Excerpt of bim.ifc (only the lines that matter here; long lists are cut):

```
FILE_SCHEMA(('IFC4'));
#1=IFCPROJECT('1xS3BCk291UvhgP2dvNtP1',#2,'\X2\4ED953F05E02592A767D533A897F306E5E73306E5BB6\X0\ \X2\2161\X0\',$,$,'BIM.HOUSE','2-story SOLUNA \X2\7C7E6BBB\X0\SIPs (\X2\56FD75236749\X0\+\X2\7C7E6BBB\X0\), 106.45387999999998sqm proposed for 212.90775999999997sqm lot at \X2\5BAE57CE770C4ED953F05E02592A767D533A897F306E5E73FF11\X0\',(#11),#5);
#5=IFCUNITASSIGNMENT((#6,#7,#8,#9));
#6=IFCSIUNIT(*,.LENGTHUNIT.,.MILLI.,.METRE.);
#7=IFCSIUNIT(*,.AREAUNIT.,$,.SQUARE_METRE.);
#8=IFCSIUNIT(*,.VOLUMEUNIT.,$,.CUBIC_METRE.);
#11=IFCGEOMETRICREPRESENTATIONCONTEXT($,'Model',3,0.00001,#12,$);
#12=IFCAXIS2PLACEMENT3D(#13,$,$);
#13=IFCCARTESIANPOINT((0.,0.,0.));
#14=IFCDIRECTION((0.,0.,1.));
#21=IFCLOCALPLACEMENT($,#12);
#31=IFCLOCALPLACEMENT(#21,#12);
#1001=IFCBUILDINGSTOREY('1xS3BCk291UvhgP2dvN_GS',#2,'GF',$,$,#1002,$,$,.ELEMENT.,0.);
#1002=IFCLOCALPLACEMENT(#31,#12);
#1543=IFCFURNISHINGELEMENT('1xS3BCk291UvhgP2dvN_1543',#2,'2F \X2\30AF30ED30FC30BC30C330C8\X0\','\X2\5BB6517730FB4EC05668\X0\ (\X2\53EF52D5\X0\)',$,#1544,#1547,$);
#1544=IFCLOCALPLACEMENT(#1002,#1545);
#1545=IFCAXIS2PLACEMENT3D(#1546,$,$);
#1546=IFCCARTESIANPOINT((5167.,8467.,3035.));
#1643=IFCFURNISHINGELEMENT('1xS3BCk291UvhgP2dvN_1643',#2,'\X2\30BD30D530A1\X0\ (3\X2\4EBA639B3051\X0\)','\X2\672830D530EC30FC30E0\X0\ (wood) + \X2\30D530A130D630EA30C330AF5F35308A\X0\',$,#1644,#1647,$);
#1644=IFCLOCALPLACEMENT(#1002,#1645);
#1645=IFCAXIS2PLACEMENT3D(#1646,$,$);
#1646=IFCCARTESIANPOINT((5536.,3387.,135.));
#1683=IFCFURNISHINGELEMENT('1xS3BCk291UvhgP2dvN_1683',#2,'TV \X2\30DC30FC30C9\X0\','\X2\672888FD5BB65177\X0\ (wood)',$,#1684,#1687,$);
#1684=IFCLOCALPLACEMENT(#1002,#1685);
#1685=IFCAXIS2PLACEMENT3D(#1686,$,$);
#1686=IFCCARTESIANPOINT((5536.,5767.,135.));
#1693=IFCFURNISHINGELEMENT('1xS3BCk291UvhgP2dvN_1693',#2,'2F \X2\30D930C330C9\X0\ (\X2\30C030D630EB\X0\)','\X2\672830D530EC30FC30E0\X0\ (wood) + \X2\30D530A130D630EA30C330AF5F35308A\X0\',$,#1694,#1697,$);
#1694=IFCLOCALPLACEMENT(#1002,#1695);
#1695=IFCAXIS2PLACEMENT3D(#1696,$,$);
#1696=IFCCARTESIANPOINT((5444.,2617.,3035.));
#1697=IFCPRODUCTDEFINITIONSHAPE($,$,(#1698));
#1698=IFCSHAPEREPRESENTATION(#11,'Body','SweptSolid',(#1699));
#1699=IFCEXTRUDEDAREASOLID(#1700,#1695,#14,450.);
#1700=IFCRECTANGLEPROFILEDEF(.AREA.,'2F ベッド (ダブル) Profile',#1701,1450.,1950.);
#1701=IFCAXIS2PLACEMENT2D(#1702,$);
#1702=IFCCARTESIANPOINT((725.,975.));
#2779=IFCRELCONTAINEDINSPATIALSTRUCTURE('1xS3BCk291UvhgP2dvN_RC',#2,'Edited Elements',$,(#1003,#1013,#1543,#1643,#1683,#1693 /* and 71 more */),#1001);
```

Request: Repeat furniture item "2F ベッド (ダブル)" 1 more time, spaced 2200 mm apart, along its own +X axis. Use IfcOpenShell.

```python
import ifcopenshell
import ifcopenshell.api.geometry
import ifcopenshell.api.root
import ifcopenshell.util.element
import ifcopenshell.util.placement

model = ifcopenshell.open("bim.ifc")


def reuse_history(source, copy):
    """copy_class also copies each property set's owner history, people and application; keep the originals."""
    for rel in copy.IsDefinedBy:
        if rel.is_a("IfcRelDefinesByProperties") and (history := rel.RelatingPropertyDefinition.OwnerHistory):
            rel.RelatingPropertyDefinition.OwnerHistory = source.OwnerHistory
            ifcopenshell.util.element.remove_deep2(model, history)


source = model.by_guid("1xS3BCk291UvhgP2dvN_1693")
base = ifcopenshell.util.placement.get_local_placement(source.ObjectPlacement)
step = base[:3, 0] * 2200.0

for i in range(1, 2):
    copy = ifcopenshell.api.root.copy_class(model, product=source)
    copy.Representation = ifcopenshell.util.element.copy_deep(
        model, source.Representation, exclude=["IfcGeometricRepresentationContext", "IfcRepresentationMap"]
    )
    reuse_history(source, copy)
    matrix = base.copy()
    matrix[:3, 3] += i * step
    print("added at", matrix[:3, 3].round(3) + 0.0)
    ifcopenshell.api.geometry.edit_object_placement(model, product=copy, matrix=matrix, is_si=False)

model.write("bim_v2.ifc")
```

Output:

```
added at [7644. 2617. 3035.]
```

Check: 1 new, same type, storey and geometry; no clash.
